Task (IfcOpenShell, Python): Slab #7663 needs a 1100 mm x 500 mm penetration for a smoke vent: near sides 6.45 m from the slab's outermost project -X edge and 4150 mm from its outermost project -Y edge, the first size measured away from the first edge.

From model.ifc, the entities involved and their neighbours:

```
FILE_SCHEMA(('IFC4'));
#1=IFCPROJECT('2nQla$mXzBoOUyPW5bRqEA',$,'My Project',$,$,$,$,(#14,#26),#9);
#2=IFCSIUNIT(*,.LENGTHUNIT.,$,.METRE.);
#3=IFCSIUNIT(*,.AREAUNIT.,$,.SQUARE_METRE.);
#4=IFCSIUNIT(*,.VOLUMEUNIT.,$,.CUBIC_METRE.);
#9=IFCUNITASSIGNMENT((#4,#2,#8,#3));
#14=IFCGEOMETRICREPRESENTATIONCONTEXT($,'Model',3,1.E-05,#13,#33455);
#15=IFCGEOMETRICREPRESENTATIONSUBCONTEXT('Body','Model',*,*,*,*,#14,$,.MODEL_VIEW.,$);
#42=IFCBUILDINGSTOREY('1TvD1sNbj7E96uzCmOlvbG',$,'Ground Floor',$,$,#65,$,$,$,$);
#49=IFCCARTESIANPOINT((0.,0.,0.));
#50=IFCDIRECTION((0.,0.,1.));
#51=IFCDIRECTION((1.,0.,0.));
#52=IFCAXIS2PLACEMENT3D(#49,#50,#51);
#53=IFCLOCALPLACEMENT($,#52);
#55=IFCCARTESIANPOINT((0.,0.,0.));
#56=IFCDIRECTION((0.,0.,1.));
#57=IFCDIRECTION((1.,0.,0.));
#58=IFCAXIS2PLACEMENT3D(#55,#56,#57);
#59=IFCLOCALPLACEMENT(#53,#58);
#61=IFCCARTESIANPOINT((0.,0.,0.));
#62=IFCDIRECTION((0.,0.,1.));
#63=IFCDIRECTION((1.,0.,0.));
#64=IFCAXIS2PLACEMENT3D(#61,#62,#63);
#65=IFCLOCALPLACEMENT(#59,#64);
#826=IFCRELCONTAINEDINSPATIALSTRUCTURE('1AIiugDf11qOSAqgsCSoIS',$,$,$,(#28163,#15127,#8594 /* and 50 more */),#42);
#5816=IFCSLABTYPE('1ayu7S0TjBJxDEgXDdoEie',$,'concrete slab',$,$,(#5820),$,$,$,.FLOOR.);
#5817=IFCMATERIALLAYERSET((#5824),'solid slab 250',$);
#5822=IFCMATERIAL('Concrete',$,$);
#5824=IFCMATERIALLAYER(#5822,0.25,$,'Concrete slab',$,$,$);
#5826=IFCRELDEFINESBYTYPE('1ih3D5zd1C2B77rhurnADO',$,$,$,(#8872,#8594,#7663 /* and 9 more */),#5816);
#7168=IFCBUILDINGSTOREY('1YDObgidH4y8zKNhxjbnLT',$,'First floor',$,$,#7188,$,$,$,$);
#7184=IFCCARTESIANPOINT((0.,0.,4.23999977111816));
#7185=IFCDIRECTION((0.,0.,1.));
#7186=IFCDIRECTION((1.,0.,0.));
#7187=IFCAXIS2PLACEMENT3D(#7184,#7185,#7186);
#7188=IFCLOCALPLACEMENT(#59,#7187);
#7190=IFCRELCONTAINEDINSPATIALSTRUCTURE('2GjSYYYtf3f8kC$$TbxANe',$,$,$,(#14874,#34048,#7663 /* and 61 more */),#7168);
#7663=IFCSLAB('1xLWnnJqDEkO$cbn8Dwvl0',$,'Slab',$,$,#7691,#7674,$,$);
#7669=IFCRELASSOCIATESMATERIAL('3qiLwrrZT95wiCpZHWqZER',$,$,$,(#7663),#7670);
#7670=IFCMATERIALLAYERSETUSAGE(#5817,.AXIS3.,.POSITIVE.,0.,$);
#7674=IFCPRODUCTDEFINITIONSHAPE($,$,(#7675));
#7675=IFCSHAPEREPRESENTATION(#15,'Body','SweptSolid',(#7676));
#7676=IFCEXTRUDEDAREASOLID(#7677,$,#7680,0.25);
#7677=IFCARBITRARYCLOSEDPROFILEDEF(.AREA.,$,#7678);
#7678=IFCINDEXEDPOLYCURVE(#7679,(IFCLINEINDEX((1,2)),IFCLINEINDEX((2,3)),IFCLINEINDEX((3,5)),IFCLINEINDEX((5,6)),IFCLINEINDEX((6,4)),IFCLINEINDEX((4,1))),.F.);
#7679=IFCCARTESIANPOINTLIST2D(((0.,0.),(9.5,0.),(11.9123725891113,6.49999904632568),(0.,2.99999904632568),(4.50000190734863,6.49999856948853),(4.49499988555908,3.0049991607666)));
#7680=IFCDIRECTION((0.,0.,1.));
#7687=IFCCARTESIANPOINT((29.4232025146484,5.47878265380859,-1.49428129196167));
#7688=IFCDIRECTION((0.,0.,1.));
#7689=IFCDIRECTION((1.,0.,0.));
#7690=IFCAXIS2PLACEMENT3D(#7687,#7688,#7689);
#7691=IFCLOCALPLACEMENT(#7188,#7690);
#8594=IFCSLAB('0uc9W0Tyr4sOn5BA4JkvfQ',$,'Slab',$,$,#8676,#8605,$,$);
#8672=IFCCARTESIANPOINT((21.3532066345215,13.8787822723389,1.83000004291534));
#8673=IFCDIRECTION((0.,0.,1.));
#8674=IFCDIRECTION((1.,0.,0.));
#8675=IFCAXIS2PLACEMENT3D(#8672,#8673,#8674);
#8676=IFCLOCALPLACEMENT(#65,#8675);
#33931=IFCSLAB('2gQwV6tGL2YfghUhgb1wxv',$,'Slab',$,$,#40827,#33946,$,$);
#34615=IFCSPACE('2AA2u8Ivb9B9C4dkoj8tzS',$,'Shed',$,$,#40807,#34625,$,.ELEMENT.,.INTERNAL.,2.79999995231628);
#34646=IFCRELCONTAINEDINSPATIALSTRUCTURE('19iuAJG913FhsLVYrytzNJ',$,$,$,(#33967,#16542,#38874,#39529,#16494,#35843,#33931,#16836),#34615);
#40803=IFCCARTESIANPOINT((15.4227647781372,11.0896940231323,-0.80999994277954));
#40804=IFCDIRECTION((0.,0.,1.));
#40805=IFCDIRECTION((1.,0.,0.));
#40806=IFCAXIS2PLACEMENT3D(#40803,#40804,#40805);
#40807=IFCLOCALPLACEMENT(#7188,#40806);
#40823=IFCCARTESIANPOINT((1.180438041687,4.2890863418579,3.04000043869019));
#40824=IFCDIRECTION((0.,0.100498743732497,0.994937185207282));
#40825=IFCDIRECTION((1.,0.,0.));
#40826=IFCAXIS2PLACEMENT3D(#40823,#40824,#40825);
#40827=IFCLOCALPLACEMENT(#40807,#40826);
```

```python
import numpy as np
import ifcopenshell
import ifcopenshell.api.feature
import ifcopenshell.api.geometry
import ifcopenshell.api.root
import ifcopenshell.geom
import ifcopenshell.util.placement
import ifcopenshell.util.representation
import ifcopenshell.util.shape
import ifcopenshell.util.unit

model = ifcopenshell.open("model.ifc")
unit_scale = ifcopenshell.util.unit.calculate_unit_scale(model)
settings = ifcopenshell.geom.settings()


def volume(element):
    """Net volume in cubic metres, openings subtracted."""
    shape = ifcopenshell.geom.create_shape(settings, element)
    return ifcopenshell.util.shape.get_volume(shape.geometry)


slab = model.by_guid("1xLWnnJqDEkO$cbn8Dwvl0")
before = volume(slab)

# Extent in the slab's own axes, in metres. The edges named are its -X and -Y sides.
slab_shape = ifcopenshell.geom.create_shape(settings, slab)
vertices = ifcopenshell.util.shape.get_vertices(slab_shape.geometry)
x_min, y_min, bottom = vertices.min(axis=0)
top = vertices[:, 2].max()

opening = ifcopenshell.api.root.create_entity(model, ifc_class="IfcOpeningElement", name="Smoke vent opening", predefined_type="OPENING")
context = ifcopenshell.util.representation.get_context(model, "Model", "Body", "MODEL_VIEW")
width, depth = 1.1, 0.5
outline = [(0.0, 0.0), (width, 0.0), (width, depth), (0.0, depth), (0.0, 0.0)]
# Overshoot both faces by 50 mm so the cut is clean.
shape = ifcopenshell.api.geometry.add_slab_representation(
    model, context=context, depth=top - bottom + 0.1, polyline=outline
)
ifcopenshell.api.geometry.assign_representation(model, product=opening, representation=shape)

matrix = ifcopenshell.util.placement.get_local_placement(slab.ObjectPlacement)
matrix[:, 3] = matrix @ np.append(np.array([x_min + 6.45, y_min + 4.15, bottom - 0.05]) / unit_scale, 1.0)
ifcopenshell.api.geometry.edit_object_placement(model, product=opening, matrix=matrix, is_si=False)
ifcopenshell.api.feature.add_feature(model, feature=opening, element=slab)

after = volume(slab)

print(f"slab volume {before:.3f} -> {after:.3f} m3")

model.write("model_rev.ifc")
```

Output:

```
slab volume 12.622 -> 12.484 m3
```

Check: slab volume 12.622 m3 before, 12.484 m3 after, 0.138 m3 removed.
